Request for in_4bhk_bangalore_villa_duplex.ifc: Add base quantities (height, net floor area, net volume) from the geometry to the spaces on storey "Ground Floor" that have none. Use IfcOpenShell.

First a look at what the model holds.

```python
import ifcopenshell
import ifcopenshell.util.element
import ifcopenshell.util.unit

model = ifcopenshell.open("in_4bhk_bangalore_villa_duplex.ifc")
print(model.schema)
for unit_type in ("LENGTHUNIT", "AREAUNIT", "VOLUMEUNIT"):
    print(unit_type, ifcopenshell.util.unit.calculate_unit_scale(model, unit_type))
storey = next(s for s in model.by_type("IfcBuildingStorey") if s.Name == "Ground Floor")
spaces = [e for e in ifcopenshell.util.element.get_decomposition(storey) if e.is_a("IfcSpace")]
for e in sorted(spaces, key=lambda e: e.id()):
    print(e.id(), e.is_a(), e.Name, list(ifcopenshell.util.element.get_psets(e, qtos_only=True)), sep=" | ")
```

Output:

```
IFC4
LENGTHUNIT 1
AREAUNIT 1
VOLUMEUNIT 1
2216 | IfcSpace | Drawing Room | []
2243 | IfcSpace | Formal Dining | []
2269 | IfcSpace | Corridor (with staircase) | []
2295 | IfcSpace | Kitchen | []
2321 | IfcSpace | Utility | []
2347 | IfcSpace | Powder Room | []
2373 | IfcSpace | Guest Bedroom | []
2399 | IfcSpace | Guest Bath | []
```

```python
import ifcopenshell
import ifcopenshell.api.pset
import ifcopenshell.geom
import ifcopenshell.util.element
import ifcopenshell.util.shape
import ifcopenshell.util.unit

model = ifcopenshell.open("in_4bhk_bangalore_villa_duplex.ifc")
unit_scale = ifcopenshell.util.unit.calculate_unit_scale(model)
area_scale = ifcopenshell.util.unit.calculate_unit_scale(model, "AREAUNIT")
volume_scale = ifcopenshell.util.unit.calculate_unit_scale(model, "VOLUMEUNIT")
settings = ifcopenshell.geom.settings()

storey = next(s for s in model.by_type("IfcBuildingStorey") if s.Name == "Ground Floor")
spaces = [e for e in ifcopenshell.util.element.get_decomposition(storey) if e.is_a("IfcSpace")]

for e in sorted(spaces, key=lambda e: e.id()):
    if ifcopenshell.util.element.get_psets(e, qtos_only=True, should_inherit=False):
        continue
    # Geometry comes back in metres, in the element's own axes.
    shape = ifcopenshell.geom.create_shape(settings, e)
    values = {
        "Height": ifcopenshell.util.shape.get_z(shape.geometry) / unit_scale,
        "NetFloorArea": ifcopenshell.util.shape.get_footprint_area(shape.geometry) / area_scale,
        "NetVolume": ifcopenshell.util.shape.get_volume(shape.geometry) / volume_scale,
    }
    qto = ifcopenshell.api.pset.add_qto(model, product=e, name="Qto_SpaceBaseQuantities")
    ifcopenshell.api.pset.edit_qto(model, qto=qto, properties=values)
    print(e.id(), {k: round(v, 3) for k, v in values.items()})

model.write("in_4bhk_bangalore_villa_duplex_updated.ifc")
```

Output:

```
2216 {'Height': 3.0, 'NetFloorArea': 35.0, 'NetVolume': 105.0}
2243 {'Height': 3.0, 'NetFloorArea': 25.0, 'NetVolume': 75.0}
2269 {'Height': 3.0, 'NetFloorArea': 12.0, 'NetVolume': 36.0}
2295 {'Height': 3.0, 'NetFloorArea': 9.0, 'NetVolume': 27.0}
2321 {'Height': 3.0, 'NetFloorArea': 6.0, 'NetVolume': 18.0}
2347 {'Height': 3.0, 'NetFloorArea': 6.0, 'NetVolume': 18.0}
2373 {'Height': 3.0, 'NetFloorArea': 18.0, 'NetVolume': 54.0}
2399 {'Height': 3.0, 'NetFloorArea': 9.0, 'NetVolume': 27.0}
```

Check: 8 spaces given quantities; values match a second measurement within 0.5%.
